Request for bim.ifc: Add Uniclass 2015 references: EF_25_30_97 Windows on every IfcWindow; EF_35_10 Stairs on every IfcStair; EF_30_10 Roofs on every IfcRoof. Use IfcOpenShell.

First a look at what the model holds.

```python
import ifcopenshell

model = ifcopenshell.open("bim.ifc")
print(model.schema)
print("classifications:", [c.Name for c in model.by_type("IfcClassification")])
for ifc_class in ("IfcDoor", "IfcRoof", "IfcStair", "IfcWall", "IfcWindow"):
    print(ifc_class, len(model.by_type(ifc_class)))
```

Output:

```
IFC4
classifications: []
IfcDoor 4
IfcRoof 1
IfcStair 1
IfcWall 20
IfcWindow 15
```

```python
import ifcopenshell
import ifcopenshell.api.classification

model = ifcopenshell.open("bim.ifc")

system = ifcopenshell.api.classification.add_classification(model, classification="Uniclass 2015")

codes = {
    "IfcWindow": ("EF_25_30_97", "Windows"),
    "IfcStair": ("EF_35_10", "Stairs"),
    "IfcRoof": ("EF_30_10", "Roofs"),
}
for ifc_class, (code, name) in codes.items():
    products = model.by_type(ifc_class)
    ifcopenshell.api.classification.add_reference(
        model, products=products, classification=system, identification=code, name=name
    )
    print(code, len(products))

model.write("bim_updated.ifc")
```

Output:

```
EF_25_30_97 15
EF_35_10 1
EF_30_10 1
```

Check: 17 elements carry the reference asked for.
